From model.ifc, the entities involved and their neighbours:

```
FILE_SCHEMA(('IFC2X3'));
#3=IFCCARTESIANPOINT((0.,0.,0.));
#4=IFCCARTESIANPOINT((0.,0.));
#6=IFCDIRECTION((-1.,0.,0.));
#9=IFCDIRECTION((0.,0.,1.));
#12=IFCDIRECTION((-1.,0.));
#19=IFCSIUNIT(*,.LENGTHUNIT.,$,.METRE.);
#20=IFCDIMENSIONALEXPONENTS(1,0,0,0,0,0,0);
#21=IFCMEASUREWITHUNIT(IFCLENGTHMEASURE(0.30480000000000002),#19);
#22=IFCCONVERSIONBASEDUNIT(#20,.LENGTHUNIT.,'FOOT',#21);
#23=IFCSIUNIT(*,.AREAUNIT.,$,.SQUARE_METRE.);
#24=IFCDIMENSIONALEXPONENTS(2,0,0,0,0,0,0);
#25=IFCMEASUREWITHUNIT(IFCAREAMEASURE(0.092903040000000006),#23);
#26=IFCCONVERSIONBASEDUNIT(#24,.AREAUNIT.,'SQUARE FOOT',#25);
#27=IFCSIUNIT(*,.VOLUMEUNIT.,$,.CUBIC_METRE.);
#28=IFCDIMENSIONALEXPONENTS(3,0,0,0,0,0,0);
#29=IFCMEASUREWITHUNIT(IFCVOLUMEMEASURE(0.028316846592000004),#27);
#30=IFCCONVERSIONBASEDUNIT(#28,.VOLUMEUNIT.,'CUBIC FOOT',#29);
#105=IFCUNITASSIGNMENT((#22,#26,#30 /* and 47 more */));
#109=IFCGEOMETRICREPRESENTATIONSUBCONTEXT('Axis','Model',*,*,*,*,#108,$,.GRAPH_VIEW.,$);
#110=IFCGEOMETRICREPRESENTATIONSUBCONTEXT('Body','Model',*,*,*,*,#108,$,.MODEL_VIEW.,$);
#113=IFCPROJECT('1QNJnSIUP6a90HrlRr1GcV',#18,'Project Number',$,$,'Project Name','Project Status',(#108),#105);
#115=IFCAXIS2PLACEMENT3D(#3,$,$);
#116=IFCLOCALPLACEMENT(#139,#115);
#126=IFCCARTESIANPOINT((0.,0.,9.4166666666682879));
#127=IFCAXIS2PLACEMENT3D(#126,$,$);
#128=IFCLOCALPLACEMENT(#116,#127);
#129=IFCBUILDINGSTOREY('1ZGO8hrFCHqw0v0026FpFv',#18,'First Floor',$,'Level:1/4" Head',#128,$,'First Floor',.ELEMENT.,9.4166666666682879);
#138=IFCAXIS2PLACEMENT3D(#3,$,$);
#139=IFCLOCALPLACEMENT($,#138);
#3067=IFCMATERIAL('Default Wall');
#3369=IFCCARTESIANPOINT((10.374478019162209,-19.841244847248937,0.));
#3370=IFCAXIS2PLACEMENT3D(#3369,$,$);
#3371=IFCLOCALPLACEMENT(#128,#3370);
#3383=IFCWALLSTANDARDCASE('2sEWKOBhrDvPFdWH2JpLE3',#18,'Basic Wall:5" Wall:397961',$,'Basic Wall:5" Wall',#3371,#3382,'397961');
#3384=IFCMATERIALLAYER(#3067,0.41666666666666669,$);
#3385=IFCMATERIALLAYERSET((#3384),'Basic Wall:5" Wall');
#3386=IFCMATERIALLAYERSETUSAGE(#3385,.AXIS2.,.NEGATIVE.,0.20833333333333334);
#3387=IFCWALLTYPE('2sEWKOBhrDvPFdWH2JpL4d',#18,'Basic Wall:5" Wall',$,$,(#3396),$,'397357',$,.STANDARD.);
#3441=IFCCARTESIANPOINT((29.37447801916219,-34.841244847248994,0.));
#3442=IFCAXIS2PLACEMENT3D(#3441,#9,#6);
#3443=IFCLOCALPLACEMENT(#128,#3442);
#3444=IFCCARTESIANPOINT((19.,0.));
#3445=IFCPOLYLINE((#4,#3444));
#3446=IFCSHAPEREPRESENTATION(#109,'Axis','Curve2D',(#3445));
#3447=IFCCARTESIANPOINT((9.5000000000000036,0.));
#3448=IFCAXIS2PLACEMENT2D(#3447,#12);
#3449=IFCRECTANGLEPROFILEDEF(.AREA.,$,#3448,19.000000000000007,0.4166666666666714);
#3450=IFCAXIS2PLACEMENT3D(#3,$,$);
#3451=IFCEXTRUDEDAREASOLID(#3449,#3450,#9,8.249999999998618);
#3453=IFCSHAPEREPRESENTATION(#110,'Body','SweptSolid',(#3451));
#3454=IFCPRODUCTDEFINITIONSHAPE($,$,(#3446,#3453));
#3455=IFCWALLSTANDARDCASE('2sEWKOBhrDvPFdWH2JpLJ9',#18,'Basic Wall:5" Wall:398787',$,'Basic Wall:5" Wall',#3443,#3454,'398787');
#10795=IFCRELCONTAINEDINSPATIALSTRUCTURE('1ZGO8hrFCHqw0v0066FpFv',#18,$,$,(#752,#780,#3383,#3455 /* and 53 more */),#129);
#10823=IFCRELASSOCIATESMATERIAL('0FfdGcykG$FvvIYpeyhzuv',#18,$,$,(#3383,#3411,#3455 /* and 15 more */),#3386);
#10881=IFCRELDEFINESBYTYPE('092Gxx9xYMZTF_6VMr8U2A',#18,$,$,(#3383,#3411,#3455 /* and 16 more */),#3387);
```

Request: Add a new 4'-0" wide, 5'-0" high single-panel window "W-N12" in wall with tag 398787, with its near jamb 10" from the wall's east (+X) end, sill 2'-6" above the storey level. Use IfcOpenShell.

```python
import numpy as np
import ifcopenshell
import ifcopenshell.api.feature
import ifcopenshell.api.geometry
import ifcopenshell.api.root
import ifcopenshell.api.spatial
import ifcopenshell.api.type
import ifcopenshell.geom
import ifcopenshell.util.element
import ifcopenshell.util.placement
import ifcopenshell.util.representation
import ifcopenshell.util.shape
import ifcopenshell.util.unit

model = ifcopenshell.open("model.ifc")
unit_scale = ifcopenshell.util.unit.calculate_unit_scale(model)
settings = ifcopenshell.geom.settings()


def volume(element):
    """Net volume in cubic metres, openings subtracted."""
    shape = ifcopenshell.geom.create_shape(settings, element)
    return ifcopenshell.util.shape.get_volume(shape.geometry)


wall = model.by_guid("2sEWKOBhrDvPFdWH2JpLJ9")
storey = ifcopenshell.util.element.get_container(wall, ifc_class="IfcBuildingStorey")
context = ifcopenshell.util.representation.get_context(model, "Model", "Body", "MODEL_VIEW")
before = volume(wall)

width, height, from_end, sill = 1.2192, 1.524, 0.254, 0.762  # metres

# The wall runs along its own X axis, and the end named is its -X end.
wall_shape = ifcopenshell.geom.create_shape(settings, wall)
x, y, z = ifcopenshell.util.shape.get_vertices(wall_shape.geometry).T
start = x.min() + from_end
face, thickness = float(y.min()), float(y.max() - y.min())
wall_matrix = ifcopenshell.util.placement.get_local_placement(wall.ObjectPlacement)
level = ifcopenshell.util.placement.get_local_placement(storey.ObjectPlacement)[2, 3]


def in_wall(x, y):
    """Placement at x, y metres in the wall's axes, at sill height."""
    matrix = wall_matrix.copy()
    matrix[:, 3] = wall_matrix @ np.array([x / unit_scale, y / unit_scale, 0.0, 1.0])
    matrix[2, 3] = level + sill / unit_scale
    return matrix


# Opening: a box that overshoots both wall faces by 50 mm.
opening = ifcopenshell.api.root.create_entity(model, ifc_class="IfcOpeningElement")
box = ifcopenshell.api.geometry.add_wall_representation(
    model, context=context, length=width, height=height, thickness=thickness + 0.1
)
ifcopenshell.api.geometry.assign_representation(model, product=opening, representation=box)
ifcopenshell.api.geometry.edit_object_placement(model, product=opening, matrix=in_wall(start, face - 0.05), is_si=False)
ifcopenshell.api.feature.add_feature(model, feature=opening, element=wall)

window = ifcopenshell.api.root.create_entity(model, ifc_class="IfcWindow", name="W-N12")
window.OverallWidth, window.OverallHeight = width / unit_scale, height / unit_scale
body = ifcopenshell.api.geometry.add_window_representation(
    model,
    context=context,
    overall_width=window.OverallWidth,
    overall_height=window.OverallHeight,
    partition_type="SINGLE_PANEL",
)
ifcopenshell.api.geometry.assign_representation(model, product=window, representation=body)
ifcopenshell.api.spatial.assign_container(model, products=[window], relating_structure=storey)
fills = ifcopenshell.api.feature.add_filling(model, opening=opening, element=window)
fills.OwnerHistory = window.OwnerHistory  # required in IFC2X3

# IFC2X3 keeps the operation on the window style.
style = ifcopenshell.api.root.create_entity(model, ifc_class="IfcWindowStyle", name="W-N12")
style.OperationType, style.ConstructionType = "SINGLE_PANEL", "NOTDEFINED"
style.ParameterTakesPrecedence = style.Sizeable = False
ifcopenshell.api.type.assign_type(model, related_objects=[window], relating_type=style)

# Centre the window in the wall's thickness.
ifcopenshell.api.geometry.edit_object_placement(model, product=window, matrix=in_wall(start, face), is_si=False)
window_shape = ifcopenshell.geom.create_shape(settings, window)
depth = ifcopenshell.util.shape.get_vertices(window_shape.geometry)[:, 1]
offset = face + thickness / 2 - (depth.min() + depth.max()) / 2
ifcopenshell.api.geometry.edit_object_placement(model, product=window, matrix=in_wall(start, offset), is_si=False)

after = volume(wall)

print(f"wall volume {before:.3f} -> {after:.3f} m3")

model.write("model_edited.ifc")
```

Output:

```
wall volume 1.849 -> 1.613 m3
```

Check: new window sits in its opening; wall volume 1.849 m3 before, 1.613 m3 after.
